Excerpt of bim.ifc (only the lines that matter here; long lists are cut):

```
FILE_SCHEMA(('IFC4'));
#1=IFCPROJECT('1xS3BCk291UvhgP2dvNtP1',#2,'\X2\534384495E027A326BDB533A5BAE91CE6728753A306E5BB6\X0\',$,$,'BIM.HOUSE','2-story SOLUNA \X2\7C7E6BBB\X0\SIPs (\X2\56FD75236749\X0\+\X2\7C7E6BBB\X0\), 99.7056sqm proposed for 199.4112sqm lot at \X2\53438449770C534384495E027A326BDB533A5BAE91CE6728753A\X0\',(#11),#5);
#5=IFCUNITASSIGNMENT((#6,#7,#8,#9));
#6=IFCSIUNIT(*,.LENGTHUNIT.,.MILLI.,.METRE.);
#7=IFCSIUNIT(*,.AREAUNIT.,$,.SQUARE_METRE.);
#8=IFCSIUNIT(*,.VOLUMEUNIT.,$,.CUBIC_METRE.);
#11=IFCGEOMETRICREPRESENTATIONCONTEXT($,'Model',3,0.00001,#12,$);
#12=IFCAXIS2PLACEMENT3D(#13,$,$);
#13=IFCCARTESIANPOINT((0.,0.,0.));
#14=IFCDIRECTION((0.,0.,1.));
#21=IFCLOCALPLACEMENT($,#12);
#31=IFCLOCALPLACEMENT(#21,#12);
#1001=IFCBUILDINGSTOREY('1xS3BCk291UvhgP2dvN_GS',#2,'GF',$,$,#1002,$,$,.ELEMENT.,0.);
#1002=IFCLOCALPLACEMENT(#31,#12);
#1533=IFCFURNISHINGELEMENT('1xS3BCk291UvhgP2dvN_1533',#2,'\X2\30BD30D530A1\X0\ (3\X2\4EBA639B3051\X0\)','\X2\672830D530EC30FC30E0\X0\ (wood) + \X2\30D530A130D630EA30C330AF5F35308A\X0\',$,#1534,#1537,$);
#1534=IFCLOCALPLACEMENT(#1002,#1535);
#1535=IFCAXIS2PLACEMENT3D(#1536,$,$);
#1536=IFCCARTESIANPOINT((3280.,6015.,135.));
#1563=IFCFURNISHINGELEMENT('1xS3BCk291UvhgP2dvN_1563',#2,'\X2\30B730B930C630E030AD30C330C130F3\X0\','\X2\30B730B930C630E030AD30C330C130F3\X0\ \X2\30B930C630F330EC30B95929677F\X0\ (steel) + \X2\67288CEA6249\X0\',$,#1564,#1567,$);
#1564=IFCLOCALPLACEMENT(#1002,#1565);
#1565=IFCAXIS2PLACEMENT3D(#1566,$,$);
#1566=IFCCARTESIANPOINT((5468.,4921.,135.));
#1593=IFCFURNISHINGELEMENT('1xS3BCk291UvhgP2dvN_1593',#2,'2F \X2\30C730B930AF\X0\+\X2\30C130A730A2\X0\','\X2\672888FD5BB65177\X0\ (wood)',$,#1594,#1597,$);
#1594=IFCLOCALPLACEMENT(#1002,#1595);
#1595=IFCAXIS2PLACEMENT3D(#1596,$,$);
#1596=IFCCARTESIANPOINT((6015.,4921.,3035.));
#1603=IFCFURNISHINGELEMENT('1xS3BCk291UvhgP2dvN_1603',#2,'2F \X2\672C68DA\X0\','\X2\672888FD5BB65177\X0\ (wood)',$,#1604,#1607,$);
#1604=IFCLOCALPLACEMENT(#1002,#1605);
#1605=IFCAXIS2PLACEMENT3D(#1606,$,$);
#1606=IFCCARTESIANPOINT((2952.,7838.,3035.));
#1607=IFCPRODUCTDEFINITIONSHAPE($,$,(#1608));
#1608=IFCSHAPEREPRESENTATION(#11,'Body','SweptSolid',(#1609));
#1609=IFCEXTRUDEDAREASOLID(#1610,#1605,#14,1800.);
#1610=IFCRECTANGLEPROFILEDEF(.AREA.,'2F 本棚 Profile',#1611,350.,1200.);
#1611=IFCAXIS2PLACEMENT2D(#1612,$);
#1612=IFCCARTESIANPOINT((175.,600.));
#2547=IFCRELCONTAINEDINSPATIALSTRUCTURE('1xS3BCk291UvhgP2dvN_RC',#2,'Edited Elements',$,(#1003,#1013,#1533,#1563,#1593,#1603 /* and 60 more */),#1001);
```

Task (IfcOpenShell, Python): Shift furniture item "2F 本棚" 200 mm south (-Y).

```python
import ifcopenshell
import ifcopenshell.api.geometry
import ifcopenshell.util.placement
import ifcopenshell.util.unit

model = ifcopenshell.open("bim.ifc")
unit_scale = ifcopenshell.util.unit.calculate_unit_scale(model)

item = model.by_guid("1xS3BCk291UvhgP2dvN_1603")
matrix = ifcopenshell.util.placement.get_local_placement(item.ObjectPlacement)
matrix[1, 3] -= 0.2 / unit_scale
ifcopenshell.api.geometry.edit_object_placement(model, product=item, matrix=matrix, is_si=False)

print(ifcopenshell.util.placement.get_local_placement(item.ObjectPlacement).round(3) + 0.0)

model.write("bim_edited.ifc")
```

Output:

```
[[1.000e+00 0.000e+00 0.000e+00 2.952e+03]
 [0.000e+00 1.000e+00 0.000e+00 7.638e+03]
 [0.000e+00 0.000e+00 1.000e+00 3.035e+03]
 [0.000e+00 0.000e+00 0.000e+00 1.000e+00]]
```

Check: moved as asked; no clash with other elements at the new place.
